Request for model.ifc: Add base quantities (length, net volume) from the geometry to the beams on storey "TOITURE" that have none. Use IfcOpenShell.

First a look at what the model holds.

```python
import ifcopenshell
import ifcopenshell.util.element
import ifcopenshell.util.unit

model = ifcopenshell.open("model.ifc")
print(model.schema)
for unit_type in ("LENGTHUNIT", "AREAUNIT", "VOLUMEUNIT"):
    print(unit_type, ifcopenshell.util.unit.calculate_unit_scale(model, unit_type))
storey = next(s for s in model.by_type("IfcBuildingStorey") if s.Name == "TOITURE")
beams = [e for e in ifcopenshell.util.element.get_decomposition(storey) if e.is_a("IfcBeam")]
for e in sorted(beams, key=lambda e: e.id()):
    print(e.id(), e.is_a(), e.Name, list(ifcopenshell.util.element.get_psets(e, qtos_only=True)), sep=" | ")
```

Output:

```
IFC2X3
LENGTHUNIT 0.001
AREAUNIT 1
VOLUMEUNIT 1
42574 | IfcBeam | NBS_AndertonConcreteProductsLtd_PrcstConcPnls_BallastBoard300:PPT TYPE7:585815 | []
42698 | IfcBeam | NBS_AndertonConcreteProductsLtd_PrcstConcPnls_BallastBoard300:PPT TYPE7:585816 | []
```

```python
import ifcopenshell
import ifcopenshell.api.pset
import ifcopenshell.geom
import ifcopenshell.util.element
import ifcopenshell.util.shape
import ifcopenshell.util.unit

model = ifcopenshell.open("model.ifc")
unit_scale = ifcopenshell.util.unit.calculate_unit_scale(model)
volume_scale = ifcopenshell.util.unit.calculate_unit_scale(model, "VOLUMEUNIT")
settings = ifcopenshell.geom.settings()

storey = next(s for s in model.by_type("IfcBuildingStorey") if s.Name == "TOITURE")
beams = [e for e in ifcopenshell.util.element.get_decomposition(storey) if e.is_a("IfcBeam")]

for e in sorted(beams, key=lambda e: e.id()):
    if ifcopenshell.util.element.get_psets(e, qtos_only=True, should_inherit=False):
        continue
    # Geometry comes back in metres, in the element's own axes.
    shape = ifcopenshell.geom.create_shape(settings, e)
    values = {
        "Length": ifcopenshell.util.shape.get_max_xyz(shape.geometry) / unit_scale,
        "NetVolume": ifcopenshell.util.shape.get_volume(shape.geometry) / volume_scale,
    }
    qto = ifcopenshell.api.pset.add_qto(model, product=e, name="BaseQuantities")
    ifcopenshell.api.pset.edit_qto(model, qto=qto, properties=values)
    print(e.id(), {k: round(v, 3) for k, v in values.items()})

model.write("model_updated.ifc")
```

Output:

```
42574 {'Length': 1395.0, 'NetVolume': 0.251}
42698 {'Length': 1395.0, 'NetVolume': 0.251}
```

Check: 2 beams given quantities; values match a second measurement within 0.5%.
